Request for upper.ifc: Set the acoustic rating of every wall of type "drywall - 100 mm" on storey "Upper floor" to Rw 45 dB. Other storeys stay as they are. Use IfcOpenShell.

First a look at what the model holds.

```python
import ifcopenshell
import ifcopenshell.util.element

model = ifcopenshell.open("upper.ifc")
print(model.schema)
storey = next(s for s in model.by_type("IfcBuildingStorey") if s.Name == "Upper floor")
walls = [e for e in ifcopenshell.util.element.get_decomposition(storey) if e.is_a("IfcWall")]
seen = {}
for e in walls:
    element_type = ifcopenshell.util.element.get_type(e)
    key = (element_type.Name if element_type != e and element_type else None, ifcopenshell.util.element.get_pset(e, "Pset_WallCommon", "AcousticRating"))
    seen[key] = seen.get(key, 0) + 1
for (name, value), count in sorted(seen.items(), key=str):
    print(count, "x", name, "|", value)
```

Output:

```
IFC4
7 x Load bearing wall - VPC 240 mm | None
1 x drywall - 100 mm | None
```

```python
import ifcopenshell
import ifcopenshell.api.pset
import ifcopenshell.util.element

model = ifcopenshell.open("upper.ifc")

storey = next(s for s in model.by_type("IfcBuildingStorey") if s.Name == "Upper floor")
walls = [e for e in ifcopenshell.util.element.get_decomposition(storey) if e.is_a("IfcWall")]

count = 0
for e in walls:
    element_type = ifcopenshell.util.element.get_type(e)
    if element_type in (None, e) or element_type.Name != "drywall - 100 mm":
        continue
    # add_pset returns the element's existing set when there is one.
    pset = ifcopenshell.api.pset.add_pset(model, product=e, name="Pset_WallCommon")
    ifcopenshell.api.pset.edit_pset(model, pset=pset, properties={"AcousticRating": "Rw 45 dB"})
    count += 1

print(count, "walls updated")

model.write("upper_updated.ifc")
```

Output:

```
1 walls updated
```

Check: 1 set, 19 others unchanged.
